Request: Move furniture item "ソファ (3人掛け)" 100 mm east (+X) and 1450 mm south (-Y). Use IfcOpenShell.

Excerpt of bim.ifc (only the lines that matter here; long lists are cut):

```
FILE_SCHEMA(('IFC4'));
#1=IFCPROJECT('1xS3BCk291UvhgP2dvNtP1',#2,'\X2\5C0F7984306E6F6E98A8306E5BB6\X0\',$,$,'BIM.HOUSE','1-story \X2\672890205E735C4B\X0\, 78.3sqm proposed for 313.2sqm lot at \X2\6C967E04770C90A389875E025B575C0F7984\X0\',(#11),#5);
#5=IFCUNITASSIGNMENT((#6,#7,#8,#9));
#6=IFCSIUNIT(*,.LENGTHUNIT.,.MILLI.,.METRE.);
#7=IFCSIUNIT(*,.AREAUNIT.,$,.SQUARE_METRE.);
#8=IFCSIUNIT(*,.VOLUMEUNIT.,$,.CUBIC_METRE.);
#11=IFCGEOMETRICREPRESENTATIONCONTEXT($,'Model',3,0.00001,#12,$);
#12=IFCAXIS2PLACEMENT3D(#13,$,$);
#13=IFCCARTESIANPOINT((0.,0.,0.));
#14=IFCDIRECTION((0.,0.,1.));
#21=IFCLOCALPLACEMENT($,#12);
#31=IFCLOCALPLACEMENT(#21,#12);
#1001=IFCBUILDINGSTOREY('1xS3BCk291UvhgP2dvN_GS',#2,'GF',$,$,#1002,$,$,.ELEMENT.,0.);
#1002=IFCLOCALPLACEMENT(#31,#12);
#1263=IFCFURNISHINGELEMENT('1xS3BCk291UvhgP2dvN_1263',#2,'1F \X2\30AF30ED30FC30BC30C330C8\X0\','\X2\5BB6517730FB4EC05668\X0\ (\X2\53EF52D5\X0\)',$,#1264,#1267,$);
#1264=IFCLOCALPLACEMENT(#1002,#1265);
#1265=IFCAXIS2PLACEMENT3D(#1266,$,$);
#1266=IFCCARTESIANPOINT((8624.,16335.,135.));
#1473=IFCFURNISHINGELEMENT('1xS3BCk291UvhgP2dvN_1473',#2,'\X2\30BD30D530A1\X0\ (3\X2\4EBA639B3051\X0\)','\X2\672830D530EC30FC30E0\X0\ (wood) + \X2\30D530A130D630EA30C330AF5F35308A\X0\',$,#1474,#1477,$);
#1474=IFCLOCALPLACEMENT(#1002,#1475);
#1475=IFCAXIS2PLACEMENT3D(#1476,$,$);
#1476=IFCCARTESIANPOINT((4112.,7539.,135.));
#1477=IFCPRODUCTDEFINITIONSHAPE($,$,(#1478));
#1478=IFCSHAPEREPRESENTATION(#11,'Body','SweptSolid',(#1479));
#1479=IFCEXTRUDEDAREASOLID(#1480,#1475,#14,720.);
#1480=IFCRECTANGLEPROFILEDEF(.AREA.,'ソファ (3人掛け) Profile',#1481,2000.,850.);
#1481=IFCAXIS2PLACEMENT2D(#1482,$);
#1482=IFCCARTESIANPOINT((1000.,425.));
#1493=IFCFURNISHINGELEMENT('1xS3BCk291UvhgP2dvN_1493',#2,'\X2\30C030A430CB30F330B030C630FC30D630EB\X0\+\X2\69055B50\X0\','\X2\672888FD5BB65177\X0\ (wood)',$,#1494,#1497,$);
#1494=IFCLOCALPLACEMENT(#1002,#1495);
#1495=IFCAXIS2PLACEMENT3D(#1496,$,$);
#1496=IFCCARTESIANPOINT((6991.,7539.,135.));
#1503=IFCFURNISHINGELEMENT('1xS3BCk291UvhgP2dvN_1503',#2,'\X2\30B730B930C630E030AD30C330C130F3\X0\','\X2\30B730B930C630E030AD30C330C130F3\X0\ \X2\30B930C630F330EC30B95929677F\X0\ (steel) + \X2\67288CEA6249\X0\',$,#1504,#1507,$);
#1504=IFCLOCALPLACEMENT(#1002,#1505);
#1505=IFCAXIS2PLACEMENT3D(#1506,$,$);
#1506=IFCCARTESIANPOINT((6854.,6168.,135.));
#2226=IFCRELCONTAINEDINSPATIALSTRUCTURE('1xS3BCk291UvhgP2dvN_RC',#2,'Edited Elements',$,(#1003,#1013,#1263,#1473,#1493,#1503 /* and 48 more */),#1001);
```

```python
import ifcopenshell
import ifcopenshell.api.geometry
import ifcopenshell.util.placement

model = ifcopenshell.open("bim.ifc")

item = model.by_guid("1xS3BCk291UvhgP2dvN_1473")
matrix = ifcopenshell.util.placement.get_local_placement(item.ObjectPlacement)
matrix[0, 3] += 100.0
matrix[1, 3] -= 1450.0
ifcopenshell.api.geometry.edit_object_placement(model, product=item, matrix=matrix, is_si=False)

print(ifcopenshell.util.placement.get_local_placement(item.ObjectPlacement).round(3) + 0.0)

model.write("bim-out.ifc")
```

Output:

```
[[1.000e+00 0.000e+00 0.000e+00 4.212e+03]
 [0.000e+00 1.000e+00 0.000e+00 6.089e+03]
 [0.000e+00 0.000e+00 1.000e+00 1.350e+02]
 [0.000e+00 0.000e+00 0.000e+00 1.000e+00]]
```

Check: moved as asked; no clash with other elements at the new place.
